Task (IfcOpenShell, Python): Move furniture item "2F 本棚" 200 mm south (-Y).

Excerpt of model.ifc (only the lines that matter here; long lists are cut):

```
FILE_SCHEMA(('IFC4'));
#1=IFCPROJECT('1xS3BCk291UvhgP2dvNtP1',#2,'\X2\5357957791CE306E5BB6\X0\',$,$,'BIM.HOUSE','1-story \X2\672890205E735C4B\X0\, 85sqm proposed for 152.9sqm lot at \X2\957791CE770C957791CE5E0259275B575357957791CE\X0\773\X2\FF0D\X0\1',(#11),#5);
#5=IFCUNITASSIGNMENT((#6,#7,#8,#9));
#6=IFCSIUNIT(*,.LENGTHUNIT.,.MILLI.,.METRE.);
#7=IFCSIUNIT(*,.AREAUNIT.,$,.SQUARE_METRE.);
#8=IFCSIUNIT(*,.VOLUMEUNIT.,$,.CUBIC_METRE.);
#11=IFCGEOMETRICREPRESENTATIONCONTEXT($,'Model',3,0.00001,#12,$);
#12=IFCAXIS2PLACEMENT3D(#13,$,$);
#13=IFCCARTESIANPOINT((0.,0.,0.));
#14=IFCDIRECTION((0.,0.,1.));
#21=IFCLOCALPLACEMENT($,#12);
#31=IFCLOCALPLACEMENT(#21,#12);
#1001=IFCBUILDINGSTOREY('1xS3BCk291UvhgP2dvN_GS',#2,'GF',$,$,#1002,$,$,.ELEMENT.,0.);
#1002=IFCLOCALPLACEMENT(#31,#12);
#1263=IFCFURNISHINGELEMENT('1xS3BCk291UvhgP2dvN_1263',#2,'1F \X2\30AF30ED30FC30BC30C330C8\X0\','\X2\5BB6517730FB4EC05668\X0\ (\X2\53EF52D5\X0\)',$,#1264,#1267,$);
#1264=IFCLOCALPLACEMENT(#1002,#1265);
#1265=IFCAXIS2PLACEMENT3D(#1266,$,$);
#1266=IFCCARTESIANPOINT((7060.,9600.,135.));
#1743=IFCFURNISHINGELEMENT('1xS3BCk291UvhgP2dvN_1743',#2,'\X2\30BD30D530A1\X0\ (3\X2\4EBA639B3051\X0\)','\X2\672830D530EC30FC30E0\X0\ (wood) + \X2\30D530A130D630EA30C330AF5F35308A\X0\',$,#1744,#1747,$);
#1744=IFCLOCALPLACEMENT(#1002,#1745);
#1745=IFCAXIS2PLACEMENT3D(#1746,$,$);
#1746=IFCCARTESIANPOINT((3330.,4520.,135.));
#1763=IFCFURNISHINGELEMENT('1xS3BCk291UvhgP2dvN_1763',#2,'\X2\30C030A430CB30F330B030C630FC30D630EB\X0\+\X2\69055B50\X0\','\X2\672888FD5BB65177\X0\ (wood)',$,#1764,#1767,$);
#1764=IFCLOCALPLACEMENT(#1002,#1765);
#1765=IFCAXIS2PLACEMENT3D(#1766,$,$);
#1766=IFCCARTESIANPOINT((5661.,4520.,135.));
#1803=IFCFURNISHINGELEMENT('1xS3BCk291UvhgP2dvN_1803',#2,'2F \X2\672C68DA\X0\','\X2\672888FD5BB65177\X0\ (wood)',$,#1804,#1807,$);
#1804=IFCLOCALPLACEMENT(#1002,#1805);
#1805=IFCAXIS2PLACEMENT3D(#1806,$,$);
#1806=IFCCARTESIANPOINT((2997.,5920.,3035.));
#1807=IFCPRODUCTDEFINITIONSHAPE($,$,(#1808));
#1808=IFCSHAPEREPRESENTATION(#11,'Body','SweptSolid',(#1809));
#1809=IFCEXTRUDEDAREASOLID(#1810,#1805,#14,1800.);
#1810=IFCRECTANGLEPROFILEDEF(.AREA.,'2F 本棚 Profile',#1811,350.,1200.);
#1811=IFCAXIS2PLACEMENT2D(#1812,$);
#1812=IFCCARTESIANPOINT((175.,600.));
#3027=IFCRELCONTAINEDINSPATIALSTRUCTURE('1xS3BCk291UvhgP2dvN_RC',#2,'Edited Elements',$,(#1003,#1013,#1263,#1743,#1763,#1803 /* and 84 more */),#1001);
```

```python
import ifcopenshell
import ifcopenshell.api.geometry
import ifcopenshell.util.placement
import ifcopenshell.util.unit

model = ifcopenshell.open("model.ifc")
unit_scale = ifcopenshell.util.unit.calculate_unit_scale(model)

item = model.by_guid("1xS3BCk291UvhgP2dvN_1803")
matrix = ifcopenshell.util.placement.get_local_placement(item.ObjectPlacement)
matrix[1, 3] -= 0.2 / unit_scale
ifcopenshell.api.geometry.edit_object_placement(model, product=item, matrix=matrix, is_si=False)

print(ifcopenshell.util.placement.get_local_placement(item.ObjectPlacement).round(3) + 0.0)

model.write("model_edited.ifc")
```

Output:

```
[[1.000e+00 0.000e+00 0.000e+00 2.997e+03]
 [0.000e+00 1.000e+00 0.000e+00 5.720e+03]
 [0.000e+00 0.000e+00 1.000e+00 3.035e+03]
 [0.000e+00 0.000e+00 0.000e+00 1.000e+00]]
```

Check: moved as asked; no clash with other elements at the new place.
